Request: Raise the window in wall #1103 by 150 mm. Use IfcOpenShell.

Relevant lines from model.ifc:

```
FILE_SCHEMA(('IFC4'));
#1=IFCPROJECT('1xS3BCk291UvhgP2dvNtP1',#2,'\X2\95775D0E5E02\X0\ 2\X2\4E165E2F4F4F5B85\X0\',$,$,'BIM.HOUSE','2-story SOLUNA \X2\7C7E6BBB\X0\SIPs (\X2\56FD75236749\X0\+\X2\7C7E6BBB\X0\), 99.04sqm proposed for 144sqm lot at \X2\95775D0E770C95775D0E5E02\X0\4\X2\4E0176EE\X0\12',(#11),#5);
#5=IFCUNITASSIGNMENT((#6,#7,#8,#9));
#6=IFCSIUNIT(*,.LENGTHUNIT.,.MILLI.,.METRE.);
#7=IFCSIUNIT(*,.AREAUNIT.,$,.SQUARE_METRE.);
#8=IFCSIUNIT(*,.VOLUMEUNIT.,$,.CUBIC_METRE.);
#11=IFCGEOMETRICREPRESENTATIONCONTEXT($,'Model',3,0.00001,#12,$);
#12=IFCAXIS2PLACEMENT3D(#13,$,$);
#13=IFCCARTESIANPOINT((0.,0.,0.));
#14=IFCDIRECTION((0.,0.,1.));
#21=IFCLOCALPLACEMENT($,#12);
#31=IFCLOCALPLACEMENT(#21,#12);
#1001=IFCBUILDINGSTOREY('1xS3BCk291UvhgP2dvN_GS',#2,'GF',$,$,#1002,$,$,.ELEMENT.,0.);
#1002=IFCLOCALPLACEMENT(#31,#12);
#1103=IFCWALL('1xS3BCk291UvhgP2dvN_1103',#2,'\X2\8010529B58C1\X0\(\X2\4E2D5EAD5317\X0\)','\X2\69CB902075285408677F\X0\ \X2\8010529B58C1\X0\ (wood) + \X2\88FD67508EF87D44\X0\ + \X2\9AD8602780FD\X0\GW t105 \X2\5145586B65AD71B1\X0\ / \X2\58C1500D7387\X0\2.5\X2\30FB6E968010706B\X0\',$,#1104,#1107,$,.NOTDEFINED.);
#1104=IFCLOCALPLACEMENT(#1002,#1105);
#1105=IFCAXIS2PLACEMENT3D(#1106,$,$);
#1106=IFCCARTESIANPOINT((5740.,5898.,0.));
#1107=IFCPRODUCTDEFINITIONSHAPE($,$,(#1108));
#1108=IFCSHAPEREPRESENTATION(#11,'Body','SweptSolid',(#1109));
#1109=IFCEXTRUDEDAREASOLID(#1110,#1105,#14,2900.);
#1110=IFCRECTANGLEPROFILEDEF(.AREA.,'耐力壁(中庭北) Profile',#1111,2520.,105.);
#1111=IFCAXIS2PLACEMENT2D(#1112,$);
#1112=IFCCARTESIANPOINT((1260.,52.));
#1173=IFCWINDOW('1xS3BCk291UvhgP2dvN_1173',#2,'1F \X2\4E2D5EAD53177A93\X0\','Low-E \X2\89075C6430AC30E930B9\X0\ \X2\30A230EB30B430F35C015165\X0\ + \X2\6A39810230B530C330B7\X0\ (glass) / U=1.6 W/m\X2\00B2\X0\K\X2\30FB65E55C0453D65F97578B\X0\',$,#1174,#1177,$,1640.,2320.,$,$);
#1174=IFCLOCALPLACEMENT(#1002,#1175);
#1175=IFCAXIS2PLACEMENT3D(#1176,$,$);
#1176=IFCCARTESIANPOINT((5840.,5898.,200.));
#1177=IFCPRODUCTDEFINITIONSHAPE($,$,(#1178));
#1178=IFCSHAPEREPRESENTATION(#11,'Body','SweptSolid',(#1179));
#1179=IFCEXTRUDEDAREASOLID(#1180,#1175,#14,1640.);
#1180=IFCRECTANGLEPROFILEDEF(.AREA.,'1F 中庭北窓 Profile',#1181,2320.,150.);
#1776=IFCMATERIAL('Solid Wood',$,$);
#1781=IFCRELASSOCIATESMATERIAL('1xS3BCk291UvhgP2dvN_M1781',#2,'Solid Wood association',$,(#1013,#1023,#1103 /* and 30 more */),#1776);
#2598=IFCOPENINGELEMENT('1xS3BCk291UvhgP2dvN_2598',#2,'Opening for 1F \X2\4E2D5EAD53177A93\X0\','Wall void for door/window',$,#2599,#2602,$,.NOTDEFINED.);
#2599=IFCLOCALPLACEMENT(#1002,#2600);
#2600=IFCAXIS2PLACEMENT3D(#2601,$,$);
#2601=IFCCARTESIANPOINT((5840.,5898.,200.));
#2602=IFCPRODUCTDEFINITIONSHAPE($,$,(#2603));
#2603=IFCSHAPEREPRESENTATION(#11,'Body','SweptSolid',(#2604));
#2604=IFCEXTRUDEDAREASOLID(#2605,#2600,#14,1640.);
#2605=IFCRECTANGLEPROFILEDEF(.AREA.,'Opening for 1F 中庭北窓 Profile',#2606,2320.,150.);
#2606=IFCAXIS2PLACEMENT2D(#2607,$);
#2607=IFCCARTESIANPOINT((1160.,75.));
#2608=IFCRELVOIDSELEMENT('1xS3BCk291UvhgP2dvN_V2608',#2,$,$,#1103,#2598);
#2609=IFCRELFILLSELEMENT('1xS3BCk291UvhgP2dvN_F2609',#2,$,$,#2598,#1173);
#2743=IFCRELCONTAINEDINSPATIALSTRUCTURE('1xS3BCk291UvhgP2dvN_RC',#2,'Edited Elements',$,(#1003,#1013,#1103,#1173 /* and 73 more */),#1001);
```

```python
import numpy as np
import ifcopenshell
import ifcopenshell.api.geometry
import ifcopenshell.util.placement
import ifcopenshell.util.unit

model = ifcopenshell.open("model.ifc")
unit_scale = ifcopenshell.util.unit.calculate_unit_scale(model)

window = model.by_guid("1xS3BCk291UvhgP2dvN_1173")
opening = window.FillsVoids[0].RelatingOpeningElement
dz = 0.15 / unit_scale

shift = np.array([0.0, 0.0, dz])
# The window is not placed relative to its opening, so move both.
for product in (opening, window):
    matrix = ifcopenshell.util.placement.get_local_placement(product.ObjectPlacement)
    matrix[:3, 3] += shift
    ifcopenshell.api.geometry.edit_object_placement(model, product=product, matrix=matrix, is_si=False)

print(f"moved by {dz * unit_scale:+.3f} m")

model.write("model_updated.ifc")
```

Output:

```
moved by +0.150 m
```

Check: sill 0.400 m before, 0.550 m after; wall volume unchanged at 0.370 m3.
